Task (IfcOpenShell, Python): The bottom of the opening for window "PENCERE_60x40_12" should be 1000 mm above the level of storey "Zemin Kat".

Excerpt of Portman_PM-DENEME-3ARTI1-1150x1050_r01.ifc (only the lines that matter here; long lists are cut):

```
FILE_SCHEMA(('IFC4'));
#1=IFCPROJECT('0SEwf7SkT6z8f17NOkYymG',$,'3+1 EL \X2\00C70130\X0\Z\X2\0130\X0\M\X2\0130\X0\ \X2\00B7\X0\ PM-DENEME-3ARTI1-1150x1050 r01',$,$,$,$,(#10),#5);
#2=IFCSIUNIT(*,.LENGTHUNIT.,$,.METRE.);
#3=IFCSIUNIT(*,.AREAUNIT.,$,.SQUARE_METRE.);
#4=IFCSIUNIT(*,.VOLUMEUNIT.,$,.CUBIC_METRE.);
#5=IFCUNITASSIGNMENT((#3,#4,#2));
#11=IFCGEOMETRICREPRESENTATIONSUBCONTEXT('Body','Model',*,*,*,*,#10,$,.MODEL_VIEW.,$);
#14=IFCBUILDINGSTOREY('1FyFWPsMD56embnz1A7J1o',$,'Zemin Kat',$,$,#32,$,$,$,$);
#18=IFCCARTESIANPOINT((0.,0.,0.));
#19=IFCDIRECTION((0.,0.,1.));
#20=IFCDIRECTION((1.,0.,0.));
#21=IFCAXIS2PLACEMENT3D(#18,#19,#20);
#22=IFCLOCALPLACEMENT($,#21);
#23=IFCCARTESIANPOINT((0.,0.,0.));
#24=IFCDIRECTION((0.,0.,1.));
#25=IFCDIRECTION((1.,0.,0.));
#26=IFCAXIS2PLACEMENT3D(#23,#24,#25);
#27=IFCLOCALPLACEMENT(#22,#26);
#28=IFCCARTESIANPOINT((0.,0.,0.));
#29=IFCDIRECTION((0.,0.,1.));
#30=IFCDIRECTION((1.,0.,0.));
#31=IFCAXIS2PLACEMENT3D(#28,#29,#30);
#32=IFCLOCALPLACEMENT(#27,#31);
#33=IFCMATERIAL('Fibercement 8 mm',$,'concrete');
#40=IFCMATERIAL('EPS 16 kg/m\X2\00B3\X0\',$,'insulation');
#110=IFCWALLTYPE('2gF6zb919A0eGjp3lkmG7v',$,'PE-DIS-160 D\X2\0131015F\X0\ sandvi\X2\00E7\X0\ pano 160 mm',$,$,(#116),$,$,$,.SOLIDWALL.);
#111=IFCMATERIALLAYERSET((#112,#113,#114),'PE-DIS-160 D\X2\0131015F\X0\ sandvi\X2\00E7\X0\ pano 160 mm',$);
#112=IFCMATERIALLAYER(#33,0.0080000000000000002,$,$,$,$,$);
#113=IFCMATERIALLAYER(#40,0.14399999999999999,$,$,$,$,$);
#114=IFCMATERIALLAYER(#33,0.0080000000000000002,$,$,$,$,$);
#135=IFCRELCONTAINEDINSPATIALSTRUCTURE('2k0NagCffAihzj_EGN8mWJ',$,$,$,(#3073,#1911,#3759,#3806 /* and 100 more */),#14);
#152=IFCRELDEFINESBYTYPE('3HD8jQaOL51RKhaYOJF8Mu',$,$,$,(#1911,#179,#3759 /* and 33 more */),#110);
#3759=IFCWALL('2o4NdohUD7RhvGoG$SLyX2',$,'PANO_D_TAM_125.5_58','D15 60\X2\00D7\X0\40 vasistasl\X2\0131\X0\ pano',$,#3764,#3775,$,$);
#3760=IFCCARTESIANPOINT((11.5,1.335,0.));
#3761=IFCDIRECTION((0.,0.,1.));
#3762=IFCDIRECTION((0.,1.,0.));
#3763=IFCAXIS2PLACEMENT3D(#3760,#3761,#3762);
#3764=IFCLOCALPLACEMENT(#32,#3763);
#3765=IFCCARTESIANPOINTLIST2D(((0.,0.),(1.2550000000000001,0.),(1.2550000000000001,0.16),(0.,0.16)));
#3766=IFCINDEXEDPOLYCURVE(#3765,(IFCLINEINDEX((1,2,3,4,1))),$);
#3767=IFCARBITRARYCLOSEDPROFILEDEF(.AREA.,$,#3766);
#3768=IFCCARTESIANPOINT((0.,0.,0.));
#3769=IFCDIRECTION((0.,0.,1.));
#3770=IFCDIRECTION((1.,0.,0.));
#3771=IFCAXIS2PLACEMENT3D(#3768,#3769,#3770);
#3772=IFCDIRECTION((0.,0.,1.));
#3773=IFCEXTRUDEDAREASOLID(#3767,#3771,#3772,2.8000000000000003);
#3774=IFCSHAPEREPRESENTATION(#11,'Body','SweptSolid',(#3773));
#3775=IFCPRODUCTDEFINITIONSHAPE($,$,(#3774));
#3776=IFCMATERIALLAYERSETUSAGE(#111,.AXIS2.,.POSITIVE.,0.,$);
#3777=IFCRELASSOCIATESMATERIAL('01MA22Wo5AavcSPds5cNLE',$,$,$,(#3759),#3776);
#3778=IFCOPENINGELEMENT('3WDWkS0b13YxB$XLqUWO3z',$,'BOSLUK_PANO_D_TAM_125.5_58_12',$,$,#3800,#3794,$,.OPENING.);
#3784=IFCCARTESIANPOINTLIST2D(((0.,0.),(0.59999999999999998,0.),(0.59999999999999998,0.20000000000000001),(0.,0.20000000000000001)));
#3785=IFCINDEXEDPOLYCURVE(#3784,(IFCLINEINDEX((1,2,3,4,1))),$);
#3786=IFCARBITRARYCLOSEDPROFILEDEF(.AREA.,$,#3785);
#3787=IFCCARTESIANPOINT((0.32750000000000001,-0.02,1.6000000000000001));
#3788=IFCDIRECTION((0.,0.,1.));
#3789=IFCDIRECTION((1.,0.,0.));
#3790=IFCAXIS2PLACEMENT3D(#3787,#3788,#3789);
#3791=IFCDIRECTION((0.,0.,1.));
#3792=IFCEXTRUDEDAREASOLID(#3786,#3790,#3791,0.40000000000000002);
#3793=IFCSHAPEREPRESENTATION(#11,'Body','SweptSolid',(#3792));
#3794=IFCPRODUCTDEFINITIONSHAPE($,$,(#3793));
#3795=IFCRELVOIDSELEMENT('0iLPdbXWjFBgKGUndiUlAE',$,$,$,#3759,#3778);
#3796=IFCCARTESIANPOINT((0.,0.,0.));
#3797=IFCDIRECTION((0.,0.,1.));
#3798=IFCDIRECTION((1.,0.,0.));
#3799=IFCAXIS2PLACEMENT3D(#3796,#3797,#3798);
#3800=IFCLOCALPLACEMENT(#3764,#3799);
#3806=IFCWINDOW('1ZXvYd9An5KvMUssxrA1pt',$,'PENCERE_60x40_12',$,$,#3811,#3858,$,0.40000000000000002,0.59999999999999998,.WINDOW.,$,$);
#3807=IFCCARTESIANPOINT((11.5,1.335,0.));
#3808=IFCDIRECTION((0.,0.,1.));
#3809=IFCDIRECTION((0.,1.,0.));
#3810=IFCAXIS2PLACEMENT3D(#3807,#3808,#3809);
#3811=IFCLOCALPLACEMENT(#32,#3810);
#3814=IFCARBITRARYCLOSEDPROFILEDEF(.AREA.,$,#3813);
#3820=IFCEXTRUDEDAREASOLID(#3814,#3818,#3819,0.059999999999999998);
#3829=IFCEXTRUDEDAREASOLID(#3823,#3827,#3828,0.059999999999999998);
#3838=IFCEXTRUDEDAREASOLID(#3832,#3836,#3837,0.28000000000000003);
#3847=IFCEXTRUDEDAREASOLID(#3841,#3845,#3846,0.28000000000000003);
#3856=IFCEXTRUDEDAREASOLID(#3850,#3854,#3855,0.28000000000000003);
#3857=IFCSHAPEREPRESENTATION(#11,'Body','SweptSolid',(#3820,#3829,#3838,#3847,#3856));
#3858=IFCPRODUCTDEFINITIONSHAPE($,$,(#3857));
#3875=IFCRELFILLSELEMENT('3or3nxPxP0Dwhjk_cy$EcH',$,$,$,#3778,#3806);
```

```python
import numpy as np
import ifcopenshell
import ifcopenshell.api.geometry
import ifcopenshell.geom
import ifcopenshell.util.element
import ifcopenshell.util.placement
import ifcopenshell.util.shape
import ifcopenshell.util.unit

model = ifcopenshell.open("Portman_PM-DENEME-3ARTI1-1150x1050_r01.ifc")
unit_scale = ifcopenshell.util.unit.calculate_unit_scale(model)

window = model.by_id(3806)
opening = window.FillsVoids[0].RelatingOpeningElement
storey = ifcopenshell.util.element.get_container(window, ifc_class="IfcBuildingStorey")
level = ifcopenshell.util.placement.get_local_placement(storey.ObjectPlacement)[2, 3]

# The opening's origin need not be at the sill, so measure its lowest point.
shape = ifcopenshell.geom.create_shape(ifcopenshell.geom.settings(), opening)
bottom = ifcopenshell.util.shape.get_shape_bottom_elevation(shape, shape.geometry) / unit_scale
dz = level + 1 / unit_scale - bottom

shift = np.array([0.0, 0.0, dz])
# The window is not placed relative to its opening, so move both.
for product in (opening, window):
    matrix = ifcopenshell.util.placement.get_local_placement(product.ObjectPlacement)
    matrix[:3, 3] += shift
    ifcopenshell.api.geometry.edit_object_placement(model, product=product, matrix=matrix, is_si=False)

print(f"moved by {dz * unit_scale:+.3f} m")

model.write("Portman_PM-DENEME-3ARTI1-1150x1050_r01_v2.ifc")
```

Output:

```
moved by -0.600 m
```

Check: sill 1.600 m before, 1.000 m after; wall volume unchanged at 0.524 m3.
